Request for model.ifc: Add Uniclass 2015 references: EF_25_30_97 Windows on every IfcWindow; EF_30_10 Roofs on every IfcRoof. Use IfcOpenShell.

First a look at what the model holds.

```python
import ifcopenshell

model = ifcopenshell.open("model.ifc")
print(model.schema)
print("classifications:", [c.Name for c in model.by_type("IfcClassification")])
for ifc_class in ("IfcDoor", "IfcRoof", "IfcStair", "IfcWall", "IfcWindow"):
    print(ifc_class, len(model.by_type(ifc_class)))
```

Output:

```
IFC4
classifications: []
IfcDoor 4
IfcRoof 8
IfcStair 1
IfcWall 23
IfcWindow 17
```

```python
import ifcopenshell
import ifcopenshell.api.classification

model = ifcopenshell.open("model.ifc")

system = ifcopenshell.api.classification.add_classification(model, classification="Uniclass 2015")

codes = {
    "IfcWindow": ("EF_25_30_97", "Windows"),
    "IfcRoof": ("EF_30_10", "Roofs"),
}
for ifc_class, (code, name) in codes.items():
    products = model.by_type(ifc_class)
    ifcopenshell.api.classification.add_reference(
        model, products=products, classification=system, identification=code, name=name
    )
    print(code, len(products))

model.write("model_v2.ifc")
```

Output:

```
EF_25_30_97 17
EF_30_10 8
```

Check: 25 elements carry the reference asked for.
